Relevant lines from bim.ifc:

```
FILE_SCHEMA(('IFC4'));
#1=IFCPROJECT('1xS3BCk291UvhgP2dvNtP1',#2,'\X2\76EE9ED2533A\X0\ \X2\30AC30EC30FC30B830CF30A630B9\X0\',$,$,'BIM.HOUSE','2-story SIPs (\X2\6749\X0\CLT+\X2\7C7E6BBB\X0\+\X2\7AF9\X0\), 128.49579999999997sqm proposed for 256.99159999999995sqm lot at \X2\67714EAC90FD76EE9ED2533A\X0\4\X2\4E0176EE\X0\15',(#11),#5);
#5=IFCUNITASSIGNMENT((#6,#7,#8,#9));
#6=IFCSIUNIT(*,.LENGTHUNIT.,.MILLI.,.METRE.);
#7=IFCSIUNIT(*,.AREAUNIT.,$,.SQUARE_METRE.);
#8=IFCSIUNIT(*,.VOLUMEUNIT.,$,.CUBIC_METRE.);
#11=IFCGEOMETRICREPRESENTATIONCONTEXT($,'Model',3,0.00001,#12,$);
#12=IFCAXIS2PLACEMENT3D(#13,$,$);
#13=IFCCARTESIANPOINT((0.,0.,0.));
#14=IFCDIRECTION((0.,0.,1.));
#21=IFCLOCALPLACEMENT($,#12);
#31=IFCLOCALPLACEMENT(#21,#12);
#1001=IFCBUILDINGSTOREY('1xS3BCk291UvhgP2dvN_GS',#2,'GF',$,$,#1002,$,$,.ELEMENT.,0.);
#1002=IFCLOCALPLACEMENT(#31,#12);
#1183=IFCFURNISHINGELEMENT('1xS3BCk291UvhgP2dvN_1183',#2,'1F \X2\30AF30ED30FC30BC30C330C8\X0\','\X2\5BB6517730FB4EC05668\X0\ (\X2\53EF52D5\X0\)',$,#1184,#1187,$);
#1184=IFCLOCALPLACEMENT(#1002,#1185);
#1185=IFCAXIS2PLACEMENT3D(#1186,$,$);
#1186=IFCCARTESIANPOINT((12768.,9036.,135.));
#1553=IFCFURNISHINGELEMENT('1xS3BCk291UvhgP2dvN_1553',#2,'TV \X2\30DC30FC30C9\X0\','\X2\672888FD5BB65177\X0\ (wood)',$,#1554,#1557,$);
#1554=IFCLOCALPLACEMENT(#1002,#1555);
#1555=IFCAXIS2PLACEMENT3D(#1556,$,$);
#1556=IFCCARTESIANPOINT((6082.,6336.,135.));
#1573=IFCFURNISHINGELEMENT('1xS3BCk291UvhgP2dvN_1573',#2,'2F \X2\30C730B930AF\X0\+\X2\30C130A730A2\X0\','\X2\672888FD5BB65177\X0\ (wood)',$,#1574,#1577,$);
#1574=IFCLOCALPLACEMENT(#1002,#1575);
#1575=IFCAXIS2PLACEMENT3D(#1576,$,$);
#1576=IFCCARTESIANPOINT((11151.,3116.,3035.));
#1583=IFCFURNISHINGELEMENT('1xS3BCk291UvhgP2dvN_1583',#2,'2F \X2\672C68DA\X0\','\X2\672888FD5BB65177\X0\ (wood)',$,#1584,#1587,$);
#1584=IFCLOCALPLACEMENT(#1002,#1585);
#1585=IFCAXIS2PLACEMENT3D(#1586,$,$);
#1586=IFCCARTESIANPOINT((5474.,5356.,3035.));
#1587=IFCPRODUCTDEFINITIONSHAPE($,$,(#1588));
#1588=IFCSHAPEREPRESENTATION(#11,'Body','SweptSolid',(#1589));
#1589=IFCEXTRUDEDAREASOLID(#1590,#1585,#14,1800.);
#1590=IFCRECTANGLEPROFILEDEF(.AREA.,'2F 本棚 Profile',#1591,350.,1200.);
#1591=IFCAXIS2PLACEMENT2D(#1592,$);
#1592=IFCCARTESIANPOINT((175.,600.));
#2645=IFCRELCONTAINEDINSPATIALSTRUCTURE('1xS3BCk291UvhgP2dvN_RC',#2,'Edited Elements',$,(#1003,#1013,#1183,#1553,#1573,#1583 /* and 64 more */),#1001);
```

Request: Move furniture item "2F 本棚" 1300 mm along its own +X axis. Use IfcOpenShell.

```python
import ifcopenshell
import ifcopenshell.api.geometry
import ifcopenshell.util.placement

model = ifcopenshell.open("bim.ifc")

item = model.by_guid("1xS3BCk291UvhgP2dvN_1583")
matrix = ifcopenshell.util.placement.get_local_placement(item.ObjectPlacement)
matrix[:3, 3] += matrix[:3, 0] * 1300.0
ifcopenshell.api.geometry.edit_object_placement(model, product=item, matrix=matrix, is_si=False)

print(ifcopenshell.util.placement.get_local_placement(item.ObjectPlacement).round(3) + 0.0)

model.write("bim_v2.ifc")
```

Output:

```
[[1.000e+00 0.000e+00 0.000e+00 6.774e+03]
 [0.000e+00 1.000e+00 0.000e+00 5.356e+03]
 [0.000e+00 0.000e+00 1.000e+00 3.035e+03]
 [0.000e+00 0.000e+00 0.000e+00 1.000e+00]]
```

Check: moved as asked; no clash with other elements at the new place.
